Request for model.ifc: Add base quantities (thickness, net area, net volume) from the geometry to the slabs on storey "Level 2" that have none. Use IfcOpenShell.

First a look at what the model holds.

```python
import ifcopenshell
import ifcopenshell.util.element
import ifcopenshell.util.unit

model = ifcopenshell.open("model.ifc")
print(model.schema)
for unit_type in ("LENGTHUNIT", "AREAUNIT", "VOLUMEUNIT"):
    print(unit_type, ifcopenshell.util.unit.calculate_unit_scale(model, unit_type))
storey = next(s for s in model.by_type("IfcBuildingStorey") if s.Name == "Level 2")
slabs = [e for e in ifcopenshell.util.element.get_decomposition(storey) if e.is_a("IfcSlab")]
for e in sorted(slabs, key=lambda e: e.id()):
    print(e.id(), e.is_a(), e.Name, list(ifcopenshell.util.element.get_psets(e, qtos_only=True)), sep=" | ")
```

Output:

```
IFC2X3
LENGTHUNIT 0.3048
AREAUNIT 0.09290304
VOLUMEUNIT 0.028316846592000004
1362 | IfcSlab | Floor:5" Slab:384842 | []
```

```python
import ifcopenshell
import ifcopenshell.api.pset
import ifcopenshell.geom
import ifcopenshell.util.element
import ifcopenshell.util.shape
import ifcopenshell.util.unit

model = ifcopenshell.open("model.ifc")
unit_scale = ifcopenshell.util.unit.calculate_unit_scale(model)
area_scale = ifcopenshell.util.unit.calculate_unit_scale(model, "AREAUNIT")
volume_scale = ifcopenshell.util.unit.calculate_unit_scale(model, "VOLUMEUNIT")
settings = ifcopenshell.geom.settings()

storey = next(s for s in model.by_type("IfcBuildingStorey") if s.Name == "Level 2")
slabs = [e for e in ifcopenshell.util.element.get_decomposition(storey) if e.is_a("IfcSlab")]

for e in sorted(slabs, key=lambda e: e.id()):
    if ifcopenshell.util.element.get_psets(e, qtos_only=True, should_inherit=False):
        continue
    # Geometry comes back in metres, in the element's own axes.
    shape = ifcopenshell.geom.create_shape(settings, e)
    values = {
        "Width": ifcopenshell.util.shape.get_z(shape.geometry) / unit_scale,
        "NetArea": ifcopenshell.util.shape.get_footprint_area(shape.geometry) / area_scale,
        "NetVolume": ifcopenshell.util.shape.get_volume(shape.geometry) / volume_scale,
    }
    qto = ifcopenshell.api.pset.add_qto(model, product=e, name="BaseQuantities")
    ifcopenshell.api.pset.edit_qto(model, qto=qto, properties=values)
    print(e.id(), {k: round(v, 3) for k, v in values.items()})

model.write("model_edited.ifc")
```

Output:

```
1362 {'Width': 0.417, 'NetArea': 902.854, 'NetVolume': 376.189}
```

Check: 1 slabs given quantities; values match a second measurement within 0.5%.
